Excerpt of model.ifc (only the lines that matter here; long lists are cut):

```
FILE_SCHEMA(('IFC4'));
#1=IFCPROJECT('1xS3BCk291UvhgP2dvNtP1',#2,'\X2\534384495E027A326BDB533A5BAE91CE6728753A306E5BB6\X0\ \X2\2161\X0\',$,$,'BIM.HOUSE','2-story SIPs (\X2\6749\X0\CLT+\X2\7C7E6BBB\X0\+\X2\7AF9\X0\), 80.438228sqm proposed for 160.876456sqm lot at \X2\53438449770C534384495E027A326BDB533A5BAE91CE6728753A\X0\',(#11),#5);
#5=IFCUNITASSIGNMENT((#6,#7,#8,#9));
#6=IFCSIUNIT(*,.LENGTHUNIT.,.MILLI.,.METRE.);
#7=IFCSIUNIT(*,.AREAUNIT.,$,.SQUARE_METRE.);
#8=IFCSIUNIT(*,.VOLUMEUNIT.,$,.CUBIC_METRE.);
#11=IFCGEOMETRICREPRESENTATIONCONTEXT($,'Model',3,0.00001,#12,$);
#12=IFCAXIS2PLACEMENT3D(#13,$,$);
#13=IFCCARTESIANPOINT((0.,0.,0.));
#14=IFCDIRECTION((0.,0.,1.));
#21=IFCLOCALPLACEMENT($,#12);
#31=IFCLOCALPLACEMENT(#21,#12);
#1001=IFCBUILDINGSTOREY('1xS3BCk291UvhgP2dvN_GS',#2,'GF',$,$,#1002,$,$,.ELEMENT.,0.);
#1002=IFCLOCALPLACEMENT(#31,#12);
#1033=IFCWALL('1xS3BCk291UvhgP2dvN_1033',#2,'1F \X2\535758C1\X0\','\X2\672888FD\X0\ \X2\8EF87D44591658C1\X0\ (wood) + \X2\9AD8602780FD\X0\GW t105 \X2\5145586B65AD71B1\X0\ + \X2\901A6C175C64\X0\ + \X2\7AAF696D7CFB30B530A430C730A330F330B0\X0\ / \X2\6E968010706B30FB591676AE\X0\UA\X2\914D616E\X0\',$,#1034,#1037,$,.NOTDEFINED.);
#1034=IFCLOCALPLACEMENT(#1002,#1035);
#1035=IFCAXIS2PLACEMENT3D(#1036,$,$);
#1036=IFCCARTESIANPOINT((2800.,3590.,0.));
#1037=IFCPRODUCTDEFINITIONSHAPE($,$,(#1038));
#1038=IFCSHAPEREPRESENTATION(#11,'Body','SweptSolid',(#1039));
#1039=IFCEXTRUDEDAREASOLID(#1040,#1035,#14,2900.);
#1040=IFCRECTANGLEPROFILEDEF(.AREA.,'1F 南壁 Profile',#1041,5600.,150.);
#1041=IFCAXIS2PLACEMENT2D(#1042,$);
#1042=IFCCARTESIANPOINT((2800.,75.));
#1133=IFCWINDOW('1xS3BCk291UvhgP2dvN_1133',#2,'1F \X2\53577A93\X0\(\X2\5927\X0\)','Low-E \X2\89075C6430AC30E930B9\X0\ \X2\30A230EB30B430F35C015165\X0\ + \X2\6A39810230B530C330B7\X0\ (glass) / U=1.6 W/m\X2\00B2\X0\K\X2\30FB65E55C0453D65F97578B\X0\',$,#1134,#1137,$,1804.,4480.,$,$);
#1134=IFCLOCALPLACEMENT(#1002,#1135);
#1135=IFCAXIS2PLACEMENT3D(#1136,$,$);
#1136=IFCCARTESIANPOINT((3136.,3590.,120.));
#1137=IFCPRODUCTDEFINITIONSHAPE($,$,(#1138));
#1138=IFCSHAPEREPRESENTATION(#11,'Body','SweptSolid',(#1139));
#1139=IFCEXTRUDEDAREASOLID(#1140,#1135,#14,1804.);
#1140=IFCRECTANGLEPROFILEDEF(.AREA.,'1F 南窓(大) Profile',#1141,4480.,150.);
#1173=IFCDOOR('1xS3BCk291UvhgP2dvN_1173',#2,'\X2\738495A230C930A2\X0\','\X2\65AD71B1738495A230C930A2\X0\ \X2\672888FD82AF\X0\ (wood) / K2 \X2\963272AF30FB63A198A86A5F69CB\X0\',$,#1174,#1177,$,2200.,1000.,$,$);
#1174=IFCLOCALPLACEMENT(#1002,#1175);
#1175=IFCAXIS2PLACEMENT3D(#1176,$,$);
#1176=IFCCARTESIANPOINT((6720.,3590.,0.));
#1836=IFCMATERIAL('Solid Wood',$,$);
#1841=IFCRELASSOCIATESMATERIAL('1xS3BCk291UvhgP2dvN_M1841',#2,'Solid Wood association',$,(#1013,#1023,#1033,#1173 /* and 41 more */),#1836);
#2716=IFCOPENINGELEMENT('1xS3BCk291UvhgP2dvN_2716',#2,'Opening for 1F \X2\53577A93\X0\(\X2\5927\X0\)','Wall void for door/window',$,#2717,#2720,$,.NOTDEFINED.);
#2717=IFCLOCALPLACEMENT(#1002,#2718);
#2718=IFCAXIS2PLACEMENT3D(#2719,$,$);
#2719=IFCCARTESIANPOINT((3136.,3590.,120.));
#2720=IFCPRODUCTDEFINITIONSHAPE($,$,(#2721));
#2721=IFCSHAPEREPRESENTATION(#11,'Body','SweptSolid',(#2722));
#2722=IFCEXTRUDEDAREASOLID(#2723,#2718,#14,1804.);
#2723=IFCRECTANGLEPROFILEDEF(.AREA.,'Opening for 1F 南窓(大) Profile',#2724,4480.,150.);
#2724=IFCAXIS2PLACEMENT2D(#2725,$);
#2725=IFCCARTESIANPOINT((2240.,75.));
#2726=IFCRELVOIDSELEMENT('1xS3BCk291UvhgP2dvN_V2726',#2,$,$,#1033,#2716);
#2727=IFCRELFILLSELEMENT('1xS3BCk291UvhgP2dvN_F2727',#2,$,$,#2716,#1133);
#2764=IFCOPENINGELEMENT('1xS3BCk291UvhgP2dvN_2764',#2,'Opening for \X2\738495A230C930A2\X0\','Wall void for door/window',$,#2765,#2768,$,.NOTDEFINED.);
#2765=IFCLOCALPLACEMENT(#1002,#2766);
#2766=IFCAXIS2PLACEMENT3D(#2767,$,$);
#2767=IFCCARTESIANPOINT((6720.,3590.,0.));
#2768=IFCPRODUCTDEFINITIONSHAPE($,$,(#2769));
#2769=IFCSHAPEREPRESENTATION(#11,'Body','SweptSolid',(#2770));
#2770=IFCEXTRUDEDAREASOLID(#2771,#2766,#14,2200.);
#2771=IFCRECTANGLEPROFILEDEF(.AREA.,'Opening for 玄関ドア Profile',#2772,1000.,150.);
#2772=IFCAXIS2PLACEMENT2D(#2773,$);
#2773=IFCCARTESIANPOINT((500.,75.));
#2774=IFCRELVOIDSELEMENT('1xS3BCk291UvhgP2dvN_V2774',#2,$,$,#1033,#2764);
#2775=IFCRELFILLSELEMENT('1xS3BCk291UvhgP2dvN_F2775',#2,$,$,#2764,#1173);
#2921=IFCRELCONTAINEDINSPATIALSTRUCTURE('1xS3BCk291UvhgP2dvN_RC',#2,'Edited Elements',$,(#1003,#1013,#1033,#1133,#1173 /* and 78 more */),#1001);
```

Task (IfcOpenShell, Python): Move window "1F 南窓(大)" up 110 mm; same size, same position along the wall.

```python
import numpy as np
import ifcopenshell
import ifcopenshell.api.geometry
import ifcopenshell.util.placement
import ifcopenshell.util.unit

model = ifcopenshell.open("model.ifc")
unit_scale = ifcopenshell.util.unit.calculate_unit_scale(model)

window = model.by_guid("1xS3BCk291UvhgP2dvN_1133")
opening = window.FillsVoids[0].RelatingOpeningElement
dz = 0.11 / unit_scale

shift = np.array([0.0, 0.0, dz])
# The window is not placed relative to its opening, so move both.
for product in (opening, window):
    matrix = ifcopenshell.util.placement.get_local_placement(product.ObjectPlacement)
    matrix[:3, 3] += shift
    ifcopenshell.api.geometry.edit_object_placement(model, product=product, matrix=matrix, is_si=False)

print(f"moved by {dz * unit_scale:+.3f} m")

model.write("model_edited.ifc")
```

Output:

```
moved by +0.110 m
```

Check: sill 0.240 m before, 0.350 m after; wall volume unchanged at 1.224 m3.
